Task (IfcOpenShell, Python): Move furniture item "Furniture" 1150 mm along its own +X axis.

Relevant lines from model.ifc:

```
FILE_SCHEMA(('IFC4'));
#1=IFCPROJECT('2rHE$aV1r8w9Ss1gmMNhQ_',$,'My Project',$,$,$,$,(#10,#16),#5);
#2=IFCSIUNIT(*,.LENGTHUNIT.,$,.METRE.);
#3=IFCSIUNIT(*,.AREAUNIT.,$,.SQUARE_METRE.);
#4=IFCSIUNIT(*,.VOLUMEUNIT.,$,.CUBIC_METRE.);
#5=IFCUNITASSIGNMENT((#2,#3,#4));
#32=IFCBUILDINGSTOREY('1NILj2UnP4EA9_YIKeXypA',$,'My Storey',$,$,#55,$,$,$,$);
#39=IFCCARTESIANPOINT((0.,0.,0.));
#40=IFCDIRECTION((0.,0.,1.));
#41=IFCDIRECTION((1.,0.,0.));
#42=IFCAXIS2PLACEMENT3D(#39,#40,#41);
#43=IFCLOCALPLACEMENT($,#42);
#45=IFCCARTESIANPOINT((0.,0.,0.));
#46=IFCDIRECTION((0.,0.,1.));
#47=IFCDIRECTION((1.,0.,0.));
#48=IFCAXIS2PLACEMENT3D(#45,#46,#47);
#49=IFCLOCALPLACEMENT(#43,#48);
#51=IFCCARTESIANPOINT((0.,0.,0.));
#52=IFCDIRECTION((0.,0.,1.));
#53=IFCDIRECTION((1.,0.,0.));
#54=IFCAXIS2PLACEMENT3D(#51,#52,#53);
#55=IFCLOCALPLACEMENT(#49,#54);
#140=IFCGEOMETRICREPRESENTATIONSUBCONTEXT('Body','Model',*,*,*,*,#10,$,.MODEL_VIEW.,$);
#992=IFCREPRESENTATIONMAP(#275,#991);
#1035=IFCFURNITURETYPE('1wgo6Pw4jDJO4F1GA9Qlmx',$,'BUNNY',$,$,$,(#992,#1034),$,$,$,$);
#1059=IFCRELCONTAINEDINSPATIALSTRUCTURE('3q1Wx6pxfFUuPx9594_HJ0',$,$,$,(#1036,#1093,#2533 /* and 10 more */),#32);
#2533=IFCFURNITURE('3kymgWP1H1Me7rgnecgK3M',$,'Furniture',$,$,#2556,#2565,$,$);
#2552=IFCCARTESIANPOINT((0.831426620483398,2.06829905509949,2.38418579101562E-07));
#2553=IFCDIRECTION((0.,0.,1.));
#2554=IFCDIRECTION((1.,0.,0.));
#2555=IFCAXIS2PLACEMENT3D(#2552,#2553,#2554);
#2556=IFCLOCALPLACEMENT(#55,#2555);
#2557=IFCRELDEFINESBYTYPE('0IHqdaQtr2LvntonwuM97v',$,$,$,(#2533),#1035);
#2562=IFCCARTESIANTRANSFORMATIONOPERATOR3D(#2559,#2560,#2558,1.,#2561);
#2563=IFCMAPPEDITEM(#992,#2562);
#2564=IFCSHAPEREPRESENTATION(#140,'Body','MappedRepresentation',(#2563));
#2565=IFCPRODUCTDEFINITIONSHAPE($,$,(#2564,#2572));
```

```python
import ifcopenshell
import ifcopenshell.api.geometry
import ifcopenshell.util.placement

model = ifcopenshell.open("model.ifc")

item = model.by_guid("3kymgWP1H1Me7rgnecgK3M")
matrix = ifcopenshell.util.placement.get_local_placement(item.ObjectPlacement)
matrix[:3, 3] += matrix[:3, 0] * 1.15
ifcopenshell.api.geometry.edit_object_placement(model, product=item, matrix=matrix, is_si=False)

print(ifcopenshell.util.placement.get_local_placement(item.ObjectPlacement).round(3) + 0.0)

model.write("model_updated.ifc")
```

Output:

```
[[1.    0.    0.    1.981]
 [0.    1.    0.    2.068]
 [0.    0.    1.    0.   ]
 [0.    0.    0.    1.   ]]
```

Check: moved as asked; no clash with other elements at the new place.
